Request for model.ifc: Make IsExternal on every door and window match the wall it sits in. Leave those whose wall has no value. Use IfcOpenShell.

First a look at what the model holds.

```python
import ifcopenshell
import ifcopenshell.util.element

model = ifcopenshell.open("model.ifc")
print(model.schema)
seen = {}
for e in model.by_type("IfcDoor") + model.by_type("IfcWindow"):
    if not e.FillsVoids:
        continue
    host = e.FillsVoids[0].RelatingOpeningElement.VoidsElements[0].RelatingBuildingElement
    own = ifcopenshell.util.element.get_pset(e, f"Pset_{e.is_a()[3:].removesuffix('StandardCase')}Common", "IsExternal")
    wall = ifcopenshell.util.element.get_pset(host, "Pset_WallCommon", "IsExternal")
    seen[e.is_a(), own, wall] = seen.get((e.is_a(), own, wall), 0) + 1
for (cls, own, wall), count in sorted(seen.items(), key=str):
    print(count, cls, "IsExternal:", own, "| host wall:", wall)
```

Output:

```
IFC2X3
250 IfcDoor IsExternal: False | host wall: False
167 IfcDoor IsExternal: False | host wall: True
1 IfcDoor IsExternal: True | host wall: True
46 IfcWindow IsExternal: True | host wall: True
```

```python
import ifcopenshell
import ifcopenshell.api.pset
import ifcopenshell.util.element

model = ifcopenshell.open("model.ifc")

count = 0
for ifc_class, pset_name in (("IfcDoor", "Pset_DoorCommon"), ("IfcWindow", "Pset_WindowCommon")):
    for e in model.by_type(ifc_class):
        if not e.FillsVoids:
            continue
        host = e.FillsVoids[0].RelatingOpeningElement.VoidsElements[0].RelatingBuildingElement
        external = ifcopenshell.util.element.get_pset(host, "Pset_WallCommon", "IsExternal")
        if external is None or ifcopenshell.util.element.get_pset(e, pset_name, "IsExternal") == external:
            continue
        pset = ifcopenshell.api.pset.add_pset(model, product=e, name=pset_name)
        ifcopenshell.api.pset.edit_pset(model, pset=pset, properties={"IsExternal": external})
        count += 1

print(count, "updated")

model.write("model_rev.ifc")
```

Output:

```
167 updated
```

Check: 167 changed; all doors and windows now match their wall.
